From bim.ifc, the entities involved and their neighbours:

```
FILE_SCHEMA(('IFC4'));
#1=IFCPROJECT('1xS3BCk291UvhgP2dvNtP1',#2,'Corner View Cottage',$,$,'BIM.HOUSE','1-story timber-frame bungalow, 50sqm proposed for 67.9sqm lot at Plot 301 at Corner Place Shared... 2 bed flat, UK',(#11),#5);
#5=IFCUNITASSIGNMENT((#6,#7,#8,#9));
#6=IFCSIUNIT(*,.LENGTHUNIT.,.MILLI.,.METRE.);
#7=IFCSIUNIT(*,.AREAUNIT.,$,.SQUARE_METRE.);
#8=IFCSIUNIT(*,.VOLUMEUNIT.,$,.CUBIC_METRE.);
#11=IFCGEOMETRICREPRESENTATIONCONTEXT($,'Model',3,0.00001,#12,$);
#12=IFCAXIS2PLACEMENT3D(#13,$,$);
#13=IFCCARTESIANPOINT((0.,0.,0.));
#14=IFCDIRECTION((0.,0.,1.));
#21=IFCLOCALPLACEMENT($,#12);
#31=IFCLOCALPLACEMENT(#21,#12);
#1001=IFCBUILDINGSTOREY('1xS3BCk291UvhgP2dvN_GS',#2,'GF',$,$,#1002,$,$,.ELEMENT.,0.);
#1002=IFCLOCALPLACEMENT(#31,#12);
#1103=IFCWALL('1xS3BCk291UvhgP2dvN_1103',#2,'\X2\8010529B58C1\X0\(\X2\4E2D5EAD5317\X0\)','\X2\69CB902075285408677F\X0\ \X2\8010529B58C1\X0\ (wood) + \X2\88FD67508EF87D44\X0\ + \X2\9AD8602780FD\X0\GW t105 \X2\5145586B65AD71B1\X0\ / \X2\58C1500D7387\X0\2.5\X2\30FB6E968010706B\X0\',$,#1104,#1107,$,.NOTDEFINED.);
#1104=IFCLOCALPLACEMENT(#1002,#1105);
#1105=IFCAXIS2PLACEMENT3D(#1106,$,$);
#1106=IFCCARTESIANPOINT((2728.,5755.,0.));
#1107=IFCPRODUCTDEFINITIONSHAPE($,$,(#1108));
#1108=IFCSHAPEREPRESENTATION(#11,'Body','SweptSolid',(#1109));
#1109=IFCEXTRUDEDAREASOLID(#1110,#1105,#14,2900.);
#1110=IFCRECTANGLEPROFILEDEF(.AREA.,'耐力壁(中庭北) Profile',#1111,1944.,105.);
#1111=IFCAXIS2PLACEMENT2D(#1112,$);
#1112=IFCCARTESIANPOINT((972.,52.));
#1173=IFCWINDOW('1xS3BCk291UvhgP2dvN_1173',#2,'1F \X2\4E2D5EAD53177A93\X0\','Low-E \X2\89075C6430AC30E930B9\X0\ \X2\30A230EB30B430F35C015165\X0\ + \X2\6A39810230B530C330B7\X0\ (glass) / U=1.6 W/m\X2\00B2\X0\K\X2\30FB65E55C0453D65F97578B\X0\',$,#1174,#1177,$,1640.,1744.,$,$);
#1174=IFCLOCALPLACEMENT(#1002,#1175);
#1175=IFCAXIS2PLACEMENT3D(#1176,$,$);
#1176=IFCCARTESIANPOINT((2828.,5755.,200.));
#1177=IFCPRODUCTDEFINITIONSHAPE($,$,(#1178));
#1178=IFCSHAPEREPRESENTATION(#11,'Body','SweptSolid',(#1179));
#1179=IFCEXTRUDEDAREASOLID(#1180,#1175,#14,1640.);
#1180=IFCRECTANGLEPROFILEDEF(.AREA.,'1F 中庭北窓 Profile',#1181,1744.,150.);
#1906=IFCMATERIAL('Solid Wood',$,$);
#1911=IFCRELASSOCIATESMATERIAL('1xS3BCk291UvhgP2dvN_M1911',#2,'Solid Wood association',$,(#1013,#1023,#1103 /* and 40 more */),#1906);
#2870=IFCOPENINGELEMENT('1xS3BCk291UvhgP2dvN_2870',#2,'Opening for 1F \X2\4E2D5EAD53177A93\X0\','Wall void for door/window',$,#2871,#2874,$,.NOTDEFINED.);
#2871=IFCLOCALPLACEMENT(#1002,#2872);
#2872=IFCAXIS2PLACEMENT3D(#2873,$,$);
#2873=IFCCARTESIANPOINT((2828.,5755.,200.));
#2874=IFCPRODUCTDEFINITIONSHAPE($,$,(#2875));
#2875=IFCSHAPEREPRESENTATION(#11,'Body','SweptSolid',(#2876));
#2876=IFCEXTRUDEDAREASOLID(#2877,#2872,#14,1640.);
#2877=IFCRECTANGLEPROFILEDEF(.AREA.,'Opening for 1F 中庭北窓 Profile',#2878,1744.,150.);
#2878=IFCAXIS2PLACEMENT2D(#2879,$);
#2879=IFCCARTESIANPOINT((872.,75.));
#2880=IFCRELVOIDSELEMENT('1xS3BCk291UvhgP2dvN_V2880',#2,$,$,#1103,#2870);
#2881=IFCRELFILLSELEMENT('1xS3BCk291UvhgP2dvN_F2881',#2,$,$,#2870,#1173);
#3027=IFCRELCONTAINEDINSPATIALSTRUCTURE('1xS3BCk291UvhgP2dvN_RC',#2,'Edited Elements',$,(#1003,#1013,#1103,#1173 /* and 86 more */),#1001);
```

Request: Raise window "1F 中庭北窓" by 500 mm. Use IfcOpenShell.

```python
import numpy as np
import ifcopenshell
import ifcopenshell.api.geometry
import ifcopenshell.util.placement
import ifcopenshell.util.unit

model = ifcopenshell.open("bim.ifc")
unit_scale = ifcopenshell.util.unit.calculate_unit_scale(model)

window = model.by_guid("1xS3BCk291UvhgP2dvN_1173")
opening = window.FillsVoids[0].RelatingOpeningElement
dz = 0.5 / unit_scale

shift = np.array([0.0, 0.0, dz])
# The window is not placed relative to its opening, so move both.
for product in (opening, window):
    matrix = ifcopenshell.util.placement.get_local_placement(product.ObjectPlacement)
    matrix[:3, 3] += shift
    ifcopenshell.api.geometry.edit_object_placement(model, product=product, matrix=matrix, is_si=False)

print(f"moved by {dz * unit_scale:+.3f} m")

model.write("bim_updated.ifc")
```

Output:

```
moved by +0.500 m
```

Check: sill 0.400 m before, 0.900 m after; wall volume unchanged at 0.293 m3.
